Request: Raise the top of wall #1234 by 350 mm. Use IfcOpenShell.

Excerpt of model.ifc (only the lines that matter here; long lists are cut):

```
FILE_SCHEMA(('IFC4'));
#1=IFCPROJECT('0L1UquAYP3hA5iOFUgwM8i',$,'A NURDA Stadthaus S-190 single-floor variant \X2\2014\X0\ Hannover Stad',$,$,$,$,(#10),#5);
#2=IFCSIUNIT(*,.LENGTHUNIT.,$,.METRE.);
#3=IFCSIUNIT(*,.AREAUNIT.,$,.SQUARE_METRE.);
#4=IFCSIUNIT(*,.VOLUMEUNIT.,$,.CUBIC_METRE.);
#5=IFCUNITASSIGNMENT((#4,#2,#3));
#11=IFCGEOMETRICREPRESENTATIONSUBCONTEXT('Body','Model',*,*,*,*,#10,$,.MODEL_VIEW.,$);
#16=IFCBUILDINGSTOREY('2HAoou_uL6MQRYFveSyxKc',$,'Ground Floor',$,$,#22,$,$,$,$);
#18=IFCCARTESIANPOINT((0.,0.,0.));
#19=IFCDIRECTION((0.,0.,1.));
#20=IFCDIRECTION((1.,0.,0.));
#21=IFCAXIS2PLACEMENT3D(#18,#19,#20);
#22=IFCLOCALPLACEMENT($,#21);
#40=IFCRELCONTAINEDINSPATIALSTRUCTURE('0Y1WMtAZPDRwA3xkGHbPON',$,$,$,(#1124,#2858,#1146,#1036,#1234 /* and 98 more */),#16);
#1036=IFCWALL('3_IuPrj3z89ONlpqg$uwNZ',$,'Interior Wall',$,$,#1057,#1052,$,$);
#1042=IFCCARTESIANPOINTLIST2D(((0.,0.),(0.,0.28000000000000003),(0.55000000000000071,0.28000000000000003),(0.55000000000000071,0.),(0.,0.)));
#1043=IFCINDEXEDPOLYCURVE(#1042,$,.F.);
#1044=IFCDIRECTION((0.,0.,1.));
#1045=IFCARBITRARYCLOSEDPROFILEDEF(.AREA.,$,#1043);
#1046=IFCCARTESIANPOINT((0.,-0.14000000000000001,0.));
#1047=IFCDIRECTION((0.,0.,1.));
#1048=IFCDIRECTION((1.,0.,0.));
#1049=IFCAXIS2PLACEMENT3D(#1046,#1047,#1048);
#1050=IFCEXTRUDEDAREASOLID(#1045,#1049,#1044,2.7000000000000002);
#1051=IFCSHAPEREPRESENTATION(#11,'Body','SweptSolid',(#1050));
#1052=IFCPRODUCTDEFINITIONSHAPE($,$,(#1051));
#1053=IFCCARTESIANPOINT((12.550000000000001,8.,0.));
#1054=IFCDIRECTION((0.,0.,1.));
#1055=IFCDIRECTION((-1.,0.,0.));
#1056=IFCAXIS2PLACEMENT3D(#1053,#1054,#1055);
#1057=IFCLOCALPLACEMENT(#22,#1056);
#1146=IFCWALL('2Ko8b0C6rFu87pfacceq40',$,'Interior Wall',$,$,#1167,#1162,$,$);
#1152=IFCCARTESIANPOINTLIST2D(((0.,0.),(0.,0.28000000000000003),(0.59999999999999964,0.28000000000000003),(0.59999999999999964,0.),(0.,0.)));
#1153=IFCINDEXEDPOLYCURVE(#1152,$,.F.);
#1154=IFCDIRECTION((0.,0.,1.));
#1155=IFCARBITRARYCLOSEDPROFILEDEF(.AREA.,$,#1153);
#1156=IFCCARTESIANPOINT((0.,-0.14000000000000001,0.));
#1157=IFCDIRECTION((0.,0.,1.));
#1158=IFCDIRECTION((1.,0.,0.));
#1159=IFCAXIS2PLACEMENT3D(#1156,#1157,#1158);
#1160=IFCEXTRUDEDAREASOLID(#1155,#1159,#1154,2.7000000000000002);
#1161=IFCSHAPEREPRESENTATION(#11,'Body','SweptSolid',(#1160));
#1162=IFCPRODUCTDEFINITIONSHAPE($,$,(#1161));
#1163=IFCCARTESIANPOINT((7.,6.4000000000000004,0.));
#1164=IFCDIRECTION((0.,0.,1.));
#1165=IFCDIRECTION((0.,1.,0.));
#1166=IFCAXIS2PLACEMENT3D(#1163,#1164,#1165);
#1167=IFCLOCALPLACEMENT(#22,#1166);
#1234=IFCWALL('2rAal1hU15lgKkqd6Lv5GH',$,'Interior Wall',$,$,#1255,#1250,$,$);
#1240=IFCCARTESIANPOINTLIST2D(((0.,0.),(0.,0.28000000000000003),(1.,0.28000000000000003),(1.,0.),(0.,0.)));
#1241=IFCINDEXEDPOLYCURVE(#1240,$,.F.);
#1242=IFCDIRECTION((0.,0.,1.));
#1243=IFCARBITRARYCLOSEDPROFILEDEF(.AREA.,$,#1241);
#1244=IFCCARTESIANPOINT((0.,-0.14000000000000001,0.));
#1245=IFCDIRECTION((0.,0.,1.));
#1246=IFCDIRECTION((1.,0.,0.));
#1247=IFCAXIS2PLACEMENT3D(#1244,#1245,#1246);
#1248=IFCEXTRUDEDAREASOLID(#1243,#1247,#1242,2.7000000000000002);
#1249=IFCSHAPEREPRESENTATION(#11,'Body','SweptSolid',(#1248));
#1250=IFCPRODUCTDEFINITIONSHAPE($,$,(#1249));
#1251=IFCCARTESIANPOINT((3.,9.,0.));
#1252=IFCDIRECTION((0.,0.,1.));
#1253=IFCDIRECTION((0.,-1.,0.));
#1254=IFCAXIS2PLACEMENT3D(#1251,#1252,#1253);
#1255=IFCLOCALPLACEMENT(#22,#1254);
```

```python
import ifcopenshell
import ifcopenshell.geom
import ifcopenshell.util.representation
import ifcopenshell.util.shape
import ifcopenshell.util.unit

model = ifcopenshell.open("model.ifc")
unit_scale = ifcopenshell.util.unit.calculate_unit_scale(model)
settings = ifcopenshell.geom.settings()


def volume(element):
    """Net volume in cubic metres, openings subtracted."""
    shape = ifcopenshell.geom.create_shape(settings, element)
    return ifcopenshell.util.shape.get_volume(shape.geometry)


wall = model.by_guid("2rAal1hU15lgKkqd6Lv5GH")
before = volume(wall)

body = ifcopenshell.util.representation.get_representation(wall, "Model", "Body")
solid = body.Items[0]
old_height = solid.Depth
solid.Depth += 0.35 / unit_scale
after = volume(wall)

print(f"height {old_height:g} -> {solid.Depth:g}, volume {before:.3f} -> {after:.3f} m3")

model.write("model_updated.ifc")
```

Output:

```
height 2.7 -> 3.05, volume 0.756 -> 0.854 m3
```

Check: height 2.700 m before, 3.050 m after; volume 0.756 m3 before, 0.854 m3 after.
